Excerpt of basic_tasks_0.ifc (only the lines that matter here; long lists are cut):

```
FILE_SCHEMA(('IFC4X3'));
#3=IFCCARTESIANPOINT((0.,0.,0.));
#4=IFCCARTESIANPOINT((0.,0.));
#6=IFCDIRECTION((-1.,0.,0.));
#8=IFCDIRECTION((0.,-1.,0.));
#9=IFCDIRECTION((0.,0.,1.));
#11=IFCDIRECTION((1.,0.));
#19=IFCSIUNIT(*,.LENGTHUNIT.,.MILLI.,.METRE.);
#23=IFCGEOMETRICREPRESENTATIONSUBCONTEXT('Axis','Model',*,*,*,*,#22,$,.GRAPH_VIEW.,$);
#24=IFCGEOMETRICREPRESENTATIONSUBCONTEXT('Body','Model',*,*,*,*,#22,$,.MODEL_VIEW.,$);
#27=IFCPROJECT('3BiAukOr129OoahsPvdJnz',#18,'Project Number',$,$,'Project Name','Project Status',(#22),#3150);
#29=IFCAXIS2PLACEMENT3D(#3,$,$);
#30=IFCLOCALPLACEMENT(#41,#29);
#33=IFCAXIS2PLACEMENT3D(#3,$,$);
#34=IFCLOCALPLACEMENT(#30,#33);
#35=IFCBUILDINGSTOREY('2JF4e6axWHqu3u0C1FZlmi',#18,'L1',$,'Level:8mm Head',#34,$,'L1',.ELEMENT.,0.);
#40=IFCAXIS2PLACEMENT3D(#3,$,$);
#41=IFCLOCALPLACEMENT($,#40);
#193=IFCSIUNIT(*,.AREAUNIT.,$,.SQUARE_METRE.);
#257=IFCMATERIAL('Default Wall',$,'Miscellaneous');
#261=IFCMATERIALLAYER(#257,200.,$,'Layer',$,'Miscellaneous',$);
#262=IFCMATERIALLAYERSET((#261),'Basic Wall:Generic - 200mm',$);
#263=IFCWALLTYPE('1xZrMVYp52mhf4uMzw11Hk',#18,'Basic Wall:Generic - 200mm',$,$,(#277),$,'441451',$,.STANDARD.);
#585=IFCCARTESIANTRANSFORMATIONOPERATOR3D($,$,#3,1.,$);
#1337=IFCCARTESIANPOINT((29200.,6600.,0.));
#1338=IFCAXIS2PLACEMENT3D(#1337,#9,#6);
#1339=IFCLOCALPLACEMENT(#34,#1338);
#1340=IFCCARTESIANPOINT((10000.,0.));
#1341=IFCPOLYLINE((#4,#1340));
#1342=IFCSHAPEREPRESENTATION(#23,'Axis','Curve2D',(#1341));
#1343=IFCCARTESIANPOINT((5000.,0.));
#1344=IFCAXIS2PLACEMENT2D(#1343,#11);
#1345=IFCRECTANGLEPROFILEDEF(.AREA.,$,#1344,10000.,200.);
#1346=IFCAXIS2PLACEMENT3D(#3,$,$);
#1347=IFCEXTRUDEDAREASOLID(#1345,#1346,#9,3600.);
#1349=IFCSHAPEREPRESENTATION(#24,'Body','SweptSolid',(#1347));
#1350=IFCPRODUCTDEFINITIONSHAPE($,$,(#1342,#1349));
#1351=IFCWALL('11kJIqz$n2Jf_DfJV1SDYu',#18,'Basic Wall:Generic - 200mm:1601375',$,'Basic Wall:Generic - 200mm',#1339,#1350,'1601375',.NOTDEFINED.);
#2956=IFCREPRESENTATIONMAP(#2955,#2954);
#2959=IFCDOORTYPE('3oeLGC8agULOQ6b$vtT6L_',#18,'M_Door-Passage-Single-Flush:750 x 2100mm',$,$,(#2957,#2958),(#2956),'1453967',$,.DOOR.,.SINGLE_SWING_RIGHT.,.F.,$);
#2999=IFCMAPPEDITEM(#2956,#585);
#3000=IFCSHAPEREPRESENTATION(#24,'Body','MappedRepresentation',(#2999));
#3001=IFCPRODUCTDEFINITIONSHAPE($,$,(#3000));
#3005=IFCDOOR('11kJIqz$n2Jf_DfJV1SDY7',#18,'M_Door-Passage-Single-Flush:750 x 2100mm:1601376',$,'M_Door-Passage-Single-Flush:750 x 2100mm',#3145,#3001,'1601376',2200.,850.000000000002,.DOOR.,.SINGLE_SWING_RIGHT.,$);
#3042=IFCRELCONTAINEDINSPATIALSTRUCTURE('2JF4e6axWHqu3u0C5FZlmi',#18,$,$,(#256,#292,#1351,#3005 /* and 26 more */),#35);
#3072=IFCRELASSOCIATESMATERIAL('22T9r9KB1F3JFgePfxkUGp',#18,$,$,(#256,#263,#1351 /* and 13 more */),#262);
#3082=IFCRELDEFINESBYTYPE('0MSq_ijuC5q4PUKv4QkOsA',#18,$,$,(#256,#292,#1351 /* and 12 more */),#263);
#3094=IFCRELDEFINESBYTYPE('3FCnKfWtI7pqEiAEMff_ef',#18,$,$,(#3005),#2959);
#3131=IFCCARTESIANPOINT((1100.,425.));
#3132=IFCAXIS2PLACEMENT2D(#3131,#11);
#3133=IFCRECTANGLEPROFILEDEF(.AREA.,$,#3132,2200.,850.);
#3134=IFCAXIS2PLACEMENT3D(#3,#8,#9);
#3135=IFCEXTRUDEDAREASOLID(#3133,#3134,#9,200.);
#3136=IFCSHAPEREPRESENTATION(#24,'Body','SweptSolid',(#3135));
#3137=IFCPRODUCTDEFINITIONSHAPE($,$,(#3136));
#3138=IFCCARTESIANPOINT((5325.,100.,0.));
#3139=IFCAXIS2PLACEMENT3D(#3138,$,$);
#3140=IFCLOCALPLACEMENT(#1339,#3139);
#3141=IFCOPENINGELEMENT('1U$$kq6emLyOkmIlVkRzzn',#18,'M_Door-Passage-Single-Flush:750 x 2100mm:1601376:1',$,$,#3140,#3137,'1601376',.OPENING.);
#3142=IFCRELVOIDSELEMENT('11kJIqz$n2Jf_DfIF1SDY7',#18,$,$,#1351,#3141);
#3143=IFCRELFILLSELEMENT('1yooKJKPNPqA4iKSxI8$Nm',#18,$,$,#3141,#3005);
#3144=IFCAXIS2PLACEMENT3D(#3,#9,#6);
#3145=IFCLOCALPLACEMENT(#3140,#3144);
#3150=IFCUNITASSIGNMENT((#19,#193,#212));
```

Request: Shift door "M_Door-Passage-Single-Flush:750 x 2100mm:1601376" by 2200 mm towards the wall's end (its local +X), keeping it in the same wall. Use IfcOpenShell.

```python
import ifcopenshell
import ifcopenshell.api.geometry
import ifcopenshell.util.placement

model = ifcopenshell.open("basic_tasks_0.ifc")

door = model.by_guid("11kJIqz$n2Jf_DfJV1SDY7")
opening = door.FillsVoids[0].RelatingOpeningElement
wall = opening.VoidsElements[0].RelatingBuildingElement

wall_matrix = ifcopenshell.util.placement.get_local_placement(wall.ObjectPlacement)
shift = wall_matrix[:3, 0] * 2200.0
before = ifcopenshell.util.placement.get_local_placement(door.ObjectPlacement)[:3, 3].copy()

# The door is placed relative to its opening, so it follows when the opening moves.
matrix = ifcopenshell.util.placement.get_local_placement(opening.ObjectPlacement)
matrix[:3, 3] += shift
ifcopenshell.api.geometry.edit_object_placement(
    model, product=opening, matrix=matrix, is_si=False, should_transform_children=True
)

after = ifcopenshell.util.placement.get_local_placement(door.ObjectPlacement)[:3, 3]
print("door moved by", (after - before).round(3) + 0.0)

model.write("basic_tasks_0_edited.ifc")
```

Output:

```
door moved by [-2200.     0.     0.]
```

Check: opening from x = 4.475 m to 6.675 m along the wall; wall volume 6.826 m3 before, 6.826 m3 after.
